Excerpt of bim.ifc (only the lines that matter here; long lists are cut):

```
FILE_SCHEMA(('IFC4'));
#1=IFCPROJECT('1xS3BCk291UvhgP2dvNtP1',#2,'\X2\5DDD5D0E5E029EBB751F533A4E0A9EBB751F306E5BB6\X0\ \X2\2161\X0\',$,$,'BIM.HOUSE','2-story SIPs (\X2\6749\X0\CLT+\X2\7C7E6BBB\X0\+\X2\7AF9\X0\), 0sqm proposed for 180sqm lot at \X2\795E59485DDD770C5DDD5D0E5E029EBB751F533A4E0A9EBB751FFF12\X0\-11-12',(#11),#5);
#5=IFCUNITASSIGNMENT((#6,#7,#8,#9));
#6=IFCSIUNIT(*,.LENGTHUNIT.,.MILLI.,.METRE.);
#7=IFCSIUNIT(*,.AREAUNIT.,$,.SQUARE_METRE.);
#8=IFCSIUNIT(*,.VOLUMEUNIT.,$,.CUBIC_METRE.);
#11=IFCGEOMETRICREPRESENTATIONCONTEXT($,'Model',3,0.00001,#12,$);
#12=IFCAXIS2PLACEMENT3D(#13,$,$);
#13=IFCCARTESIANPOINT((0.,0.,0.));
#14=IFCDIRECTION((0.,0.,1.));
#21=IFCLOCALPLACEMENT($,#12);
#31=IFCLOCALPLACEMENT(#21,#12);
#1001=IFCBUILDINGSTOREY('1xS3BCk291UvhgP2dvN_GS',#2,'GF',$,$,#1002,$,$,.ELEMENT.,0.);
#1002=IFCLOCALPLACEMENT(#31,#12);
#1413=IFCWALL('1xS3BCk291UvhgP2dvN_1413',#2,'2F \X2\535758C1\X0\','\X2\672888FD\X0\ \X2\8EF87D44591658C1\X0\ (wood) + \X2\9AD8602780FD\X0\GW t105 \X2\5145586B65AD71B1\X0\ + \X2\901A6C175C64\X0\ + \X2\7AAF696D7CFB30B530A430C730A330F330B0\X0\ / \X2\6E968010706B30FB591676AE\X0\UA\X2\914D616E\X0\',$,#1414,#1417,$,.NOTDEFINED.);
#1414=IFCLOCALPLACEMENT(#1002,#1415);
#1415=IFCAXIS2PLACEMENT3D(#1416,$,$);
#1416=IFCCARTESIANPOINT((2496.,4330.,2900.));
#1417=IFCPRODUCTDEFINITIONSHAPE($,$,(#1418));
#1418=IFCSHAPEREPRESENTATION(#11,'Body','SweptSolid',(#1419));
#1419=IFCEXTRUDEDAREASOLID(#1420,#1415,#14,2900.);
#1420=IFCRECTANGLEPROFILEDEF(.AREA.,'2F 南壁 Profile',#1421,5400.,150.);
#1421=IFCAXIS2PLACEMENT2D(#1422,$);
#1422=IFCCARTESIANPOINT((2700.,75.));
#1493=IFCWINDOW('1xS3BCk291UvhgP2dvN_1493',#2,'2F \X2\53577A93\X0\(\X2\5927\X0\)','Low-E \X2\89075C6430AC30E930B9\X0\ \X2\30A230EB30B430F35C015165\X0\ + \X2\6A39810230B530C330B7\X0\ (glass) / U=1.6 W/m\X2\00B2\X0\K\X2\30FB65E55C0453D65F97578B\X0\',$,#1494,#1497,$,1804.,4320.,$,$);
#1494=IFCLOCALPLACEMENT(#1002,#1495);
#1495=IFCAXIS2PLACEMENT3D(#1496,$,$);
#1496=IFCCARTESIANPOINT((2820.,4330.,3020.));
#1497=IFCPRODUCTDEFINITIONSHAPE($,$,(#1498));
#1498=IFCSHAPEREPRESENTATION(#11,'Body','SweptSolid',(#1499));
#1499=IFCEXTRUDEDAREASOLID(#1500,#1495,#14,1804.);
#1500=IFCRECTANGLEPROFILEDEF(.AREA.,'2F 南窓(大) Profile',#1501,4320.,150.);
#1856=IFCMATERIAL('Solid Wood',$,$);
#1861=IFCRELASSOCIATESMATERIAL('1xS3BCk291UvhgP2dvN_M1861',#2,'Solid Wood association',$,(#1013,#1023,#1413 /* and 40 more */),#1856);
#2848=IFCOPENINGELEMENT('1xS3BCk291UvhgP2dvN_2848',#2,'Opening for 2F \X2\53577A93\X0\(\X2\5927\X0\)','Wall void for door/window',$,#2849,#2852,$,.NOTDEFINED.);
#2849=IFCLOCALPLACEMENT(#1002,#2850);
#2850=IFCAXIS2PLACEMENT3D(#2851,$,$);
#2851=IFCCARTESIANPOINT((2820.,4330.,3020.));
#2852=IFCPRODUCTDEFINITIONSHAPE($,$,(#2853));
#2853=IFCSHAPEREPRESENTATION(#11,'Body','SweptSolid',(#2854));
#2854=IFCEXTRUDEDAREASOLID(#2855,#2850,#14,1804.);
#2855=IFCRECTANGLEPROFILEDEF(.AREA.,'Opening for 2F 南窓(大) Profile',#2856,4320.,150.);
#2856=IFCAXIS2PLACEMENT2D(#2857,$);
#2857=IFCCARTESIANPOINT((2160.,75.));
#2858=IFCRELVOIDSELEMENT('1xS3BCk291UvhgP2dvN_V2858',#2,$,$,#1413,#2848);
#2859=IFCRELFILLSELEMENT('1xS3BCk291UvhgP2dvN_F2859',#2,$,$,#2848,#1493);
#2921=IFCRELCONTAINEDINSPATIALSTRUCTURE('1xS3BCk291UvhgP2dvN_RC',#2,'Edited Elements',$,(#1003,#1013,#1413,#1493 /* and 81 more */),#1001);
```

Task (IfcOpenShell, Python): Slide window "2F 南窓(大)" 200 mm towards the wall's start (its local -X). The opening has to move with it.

```python
import ifcopenshell
import ifcopenshell.api.geometry
import ifcopenshell.util.placement
import ifcopenshell.util.unit

model = ifcopenshell.open("bim.ifc")
unit_scale = ifcopenshell.util.unit.calculate_unit_scale(model)

window = model.by_id(1493)
opening = window.FillsVoids[0].RelatingOpeningElement
wall = opening.VoidsElements[0].RelatingBuildingElement

wall_matrix = ifcopenshell.util.placement.get_local_placement(wall.ObjectPlacement)
shift = wall_matrix[:3, 0] * -0.2 / unit_scale
before = ifcopenshell.util.placement.get_local_placement(window.ObjectPlacement)[:3, 3].copy()

# The window is not placed relative to its opening, so move both.
for product in (opening, window):
    matrix = ifcopenshell.util.placement.get_local_placement(product.ObjectPlacement)
    matrix[:3, 3] += shift
    ifcopenshell.api.geometry.edit_object_placement(model, product=product, matrix=matrix, is_si=False)

after = ifcopenshell.util.placement.get_local_placement(window.ObjectPlacement)[:3, 3]
print("window moved by", (after - before).round(3) + 0.0)

model.write("bim_rev.ifc")
```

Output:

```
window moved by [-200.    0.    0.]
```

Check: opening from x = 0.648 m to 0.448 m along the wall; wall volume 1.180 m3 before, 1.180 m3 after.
